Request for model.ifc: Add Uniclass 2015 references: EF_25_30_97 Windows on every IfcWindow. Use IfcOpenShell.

First a look at what the model holds.

```python
import ifcopenshell

model = ifcopenshell.open("model.ifc")
print(model.schema)
print("classifications:", [c.Name for c in model.by_type("IfcClassification")])
for ifc_class in ("IfcDoor", "IfcRoof", "IfcStair", "IfcWall", "IfcWindow"):
    print(ifc_class, len(model.by_type(ifc_class)))
```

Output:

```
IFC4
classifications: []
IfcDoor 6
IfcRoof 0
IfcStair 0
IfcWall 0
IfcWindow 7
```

```python
import ifcopenshell
import ifcopenshell.api.classification

model = ifcopenshell.open("model.ifc")

system = ifcopenshell.api.classification.add_classification(model, classification="Uniclass 2015")

codes = {
    "IfcWindow": ("EF_25_30_97", "Windows"),
}
for ifc_class, (code, name) in codes.items():
    products = model.by_type(ifc_class)
    ifcopenshell.api.classification.add_reference(
        model, products=products, classification=system, identification=code, name=name
    )
    print(code, len(products))

model.write("model_updated.ifc")
```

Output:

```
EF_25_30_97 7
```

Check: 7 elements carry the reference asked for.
